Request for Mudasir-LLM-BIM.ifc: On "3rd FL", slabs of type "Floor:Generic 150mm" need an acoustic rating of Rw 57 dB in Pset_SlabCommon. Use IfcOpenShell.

First a look at what the model holds.

```python
import ifcopenshell
import ifcopenshell.util.element

model = ifcopenshell.open("Mudasir-LLM-BIM.ifc")
print(model.schema)
storey = next(s for s in model.by_type("IfcBuildingStorey") if s.Name == "3rd FL")
slabs = [e for e in ifcopenshell.util.element.get_decomposition(storey) if e.is_a("IfcSlab")]
seen = {}
for e in slabs:
    element_type = ifcopenshell.util.element.get_type(e)
    key = (element_type.Name if element_type != e and element_type else None, ifcopenshell.util.element.get_pset(e, "Pset_SlabCommon", "AcousticRating"))
    seen[key] = seen.get(key, 0) + 1
for (name, value), count in sorted(seen.items(), key=str):
    print(count, "x", name, "|", value)
```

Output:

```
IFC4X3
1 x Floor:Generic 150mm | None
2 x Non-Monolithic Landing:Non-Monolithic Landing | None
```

```python
import ifcopenshell
import ifcopenshell.api.pset
import ifcopenshell.util.element

model = ifcopenshell.open("Mudasir-LLM-BIM.ifc")

storey = next(s for s in model.by_type("IfcBuildingStorey") if s.Name == "3rd FL")
slabs = [e for e in ifcopenshell.util.element.get_decomposition(storey) if e.is_a("IfcSlab")]

count = 0
for e in slabs:
    element_type = ifcopenshell.util.element.get_type(e)
    if element_type in (None, e) or element_type.Name != "Floor:Generic 150mm":
        continue
    # add_pset returns the element's existing set when there is one.
    pset = ifcopenshell.api.pset.add_pset(model, product=e, name="Pset_SlabCommon")
    ifcopenshell.api.pset.edit_pset(model, pset=pset, properties={"AcousticRating": "Rw 57 dB"})
    count += 1

print(count, "slabs updated")

model.write("Mudasir-LLM-BIM_updated.ifc")
```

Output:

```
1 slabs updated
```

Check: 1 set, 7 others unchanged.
